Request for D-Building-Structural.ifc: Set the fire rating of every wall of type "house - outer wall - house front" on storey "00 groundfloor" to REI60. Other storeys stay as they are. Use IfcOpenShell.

First a look at what the model holds.

```python
import ifcopenshell
import ifcopenshell.util.element

model = ifcopenshell.open("D-Building-Structural.ifc")
print(model.schema)
storey = next(s for s in model.by_type("IfcBuildingStorey") if s.Name == "00 groundfloor")
walls = [e for e in ifcopenshell.util.element.get_decomposition(storey) if e.is_a("IfcWall")]
seen = {}
for e in walls:
    element_type = ifcopenshell.util.element.get_type(e)
    key = (element_type.Name if element_type != e and element_type else None, ifcopenshell.util.element.get_pset(e, "Pset_WallCommon", "FireRating"))
    seen[key] = seen.get(key, 0) + 1
for (name, value), count in sorted(seen.items(), key=str):
    print(count, "x", name, "|", value)
```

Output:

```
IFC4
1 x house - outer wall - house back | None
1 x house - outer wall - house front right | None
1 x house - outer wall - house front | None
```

```python
import ifcopenshell
import ifcopenshell.api.pset
import ifcopenshell.util.element

model = ifcopenshell.open("D-Building-Structural.ifc")

storey = next(s for s in model.by_type("IfcBuildingStorey") if s.Name == "00 groundfloor")
walls = [e for e in ifcopenshell.util.element.get_decomposition(storey) if e.is_a("IfcWall")]

count = 0
for e in walls:
    element_type = ifcopenshell.util.element.get_type(e)
    if element_type in (None, e) or element_type.Name != "house - outer wall - house front":
        continue
    # add_pset returns the element's existing set when there is one.
    pset = ifcopenshell.api.pset.add_pset(model, product=e, name="Pset_WallCommon")
    ifcopenshell.api.pset.edit_pset(model, pset=pset, properties={"FireRating": "REI60"})
    count += 1

print(count, "walls updated")

model.write("D-Building-Structural_edited.ifc")
```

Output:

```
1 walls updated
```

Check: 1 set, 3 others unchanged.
